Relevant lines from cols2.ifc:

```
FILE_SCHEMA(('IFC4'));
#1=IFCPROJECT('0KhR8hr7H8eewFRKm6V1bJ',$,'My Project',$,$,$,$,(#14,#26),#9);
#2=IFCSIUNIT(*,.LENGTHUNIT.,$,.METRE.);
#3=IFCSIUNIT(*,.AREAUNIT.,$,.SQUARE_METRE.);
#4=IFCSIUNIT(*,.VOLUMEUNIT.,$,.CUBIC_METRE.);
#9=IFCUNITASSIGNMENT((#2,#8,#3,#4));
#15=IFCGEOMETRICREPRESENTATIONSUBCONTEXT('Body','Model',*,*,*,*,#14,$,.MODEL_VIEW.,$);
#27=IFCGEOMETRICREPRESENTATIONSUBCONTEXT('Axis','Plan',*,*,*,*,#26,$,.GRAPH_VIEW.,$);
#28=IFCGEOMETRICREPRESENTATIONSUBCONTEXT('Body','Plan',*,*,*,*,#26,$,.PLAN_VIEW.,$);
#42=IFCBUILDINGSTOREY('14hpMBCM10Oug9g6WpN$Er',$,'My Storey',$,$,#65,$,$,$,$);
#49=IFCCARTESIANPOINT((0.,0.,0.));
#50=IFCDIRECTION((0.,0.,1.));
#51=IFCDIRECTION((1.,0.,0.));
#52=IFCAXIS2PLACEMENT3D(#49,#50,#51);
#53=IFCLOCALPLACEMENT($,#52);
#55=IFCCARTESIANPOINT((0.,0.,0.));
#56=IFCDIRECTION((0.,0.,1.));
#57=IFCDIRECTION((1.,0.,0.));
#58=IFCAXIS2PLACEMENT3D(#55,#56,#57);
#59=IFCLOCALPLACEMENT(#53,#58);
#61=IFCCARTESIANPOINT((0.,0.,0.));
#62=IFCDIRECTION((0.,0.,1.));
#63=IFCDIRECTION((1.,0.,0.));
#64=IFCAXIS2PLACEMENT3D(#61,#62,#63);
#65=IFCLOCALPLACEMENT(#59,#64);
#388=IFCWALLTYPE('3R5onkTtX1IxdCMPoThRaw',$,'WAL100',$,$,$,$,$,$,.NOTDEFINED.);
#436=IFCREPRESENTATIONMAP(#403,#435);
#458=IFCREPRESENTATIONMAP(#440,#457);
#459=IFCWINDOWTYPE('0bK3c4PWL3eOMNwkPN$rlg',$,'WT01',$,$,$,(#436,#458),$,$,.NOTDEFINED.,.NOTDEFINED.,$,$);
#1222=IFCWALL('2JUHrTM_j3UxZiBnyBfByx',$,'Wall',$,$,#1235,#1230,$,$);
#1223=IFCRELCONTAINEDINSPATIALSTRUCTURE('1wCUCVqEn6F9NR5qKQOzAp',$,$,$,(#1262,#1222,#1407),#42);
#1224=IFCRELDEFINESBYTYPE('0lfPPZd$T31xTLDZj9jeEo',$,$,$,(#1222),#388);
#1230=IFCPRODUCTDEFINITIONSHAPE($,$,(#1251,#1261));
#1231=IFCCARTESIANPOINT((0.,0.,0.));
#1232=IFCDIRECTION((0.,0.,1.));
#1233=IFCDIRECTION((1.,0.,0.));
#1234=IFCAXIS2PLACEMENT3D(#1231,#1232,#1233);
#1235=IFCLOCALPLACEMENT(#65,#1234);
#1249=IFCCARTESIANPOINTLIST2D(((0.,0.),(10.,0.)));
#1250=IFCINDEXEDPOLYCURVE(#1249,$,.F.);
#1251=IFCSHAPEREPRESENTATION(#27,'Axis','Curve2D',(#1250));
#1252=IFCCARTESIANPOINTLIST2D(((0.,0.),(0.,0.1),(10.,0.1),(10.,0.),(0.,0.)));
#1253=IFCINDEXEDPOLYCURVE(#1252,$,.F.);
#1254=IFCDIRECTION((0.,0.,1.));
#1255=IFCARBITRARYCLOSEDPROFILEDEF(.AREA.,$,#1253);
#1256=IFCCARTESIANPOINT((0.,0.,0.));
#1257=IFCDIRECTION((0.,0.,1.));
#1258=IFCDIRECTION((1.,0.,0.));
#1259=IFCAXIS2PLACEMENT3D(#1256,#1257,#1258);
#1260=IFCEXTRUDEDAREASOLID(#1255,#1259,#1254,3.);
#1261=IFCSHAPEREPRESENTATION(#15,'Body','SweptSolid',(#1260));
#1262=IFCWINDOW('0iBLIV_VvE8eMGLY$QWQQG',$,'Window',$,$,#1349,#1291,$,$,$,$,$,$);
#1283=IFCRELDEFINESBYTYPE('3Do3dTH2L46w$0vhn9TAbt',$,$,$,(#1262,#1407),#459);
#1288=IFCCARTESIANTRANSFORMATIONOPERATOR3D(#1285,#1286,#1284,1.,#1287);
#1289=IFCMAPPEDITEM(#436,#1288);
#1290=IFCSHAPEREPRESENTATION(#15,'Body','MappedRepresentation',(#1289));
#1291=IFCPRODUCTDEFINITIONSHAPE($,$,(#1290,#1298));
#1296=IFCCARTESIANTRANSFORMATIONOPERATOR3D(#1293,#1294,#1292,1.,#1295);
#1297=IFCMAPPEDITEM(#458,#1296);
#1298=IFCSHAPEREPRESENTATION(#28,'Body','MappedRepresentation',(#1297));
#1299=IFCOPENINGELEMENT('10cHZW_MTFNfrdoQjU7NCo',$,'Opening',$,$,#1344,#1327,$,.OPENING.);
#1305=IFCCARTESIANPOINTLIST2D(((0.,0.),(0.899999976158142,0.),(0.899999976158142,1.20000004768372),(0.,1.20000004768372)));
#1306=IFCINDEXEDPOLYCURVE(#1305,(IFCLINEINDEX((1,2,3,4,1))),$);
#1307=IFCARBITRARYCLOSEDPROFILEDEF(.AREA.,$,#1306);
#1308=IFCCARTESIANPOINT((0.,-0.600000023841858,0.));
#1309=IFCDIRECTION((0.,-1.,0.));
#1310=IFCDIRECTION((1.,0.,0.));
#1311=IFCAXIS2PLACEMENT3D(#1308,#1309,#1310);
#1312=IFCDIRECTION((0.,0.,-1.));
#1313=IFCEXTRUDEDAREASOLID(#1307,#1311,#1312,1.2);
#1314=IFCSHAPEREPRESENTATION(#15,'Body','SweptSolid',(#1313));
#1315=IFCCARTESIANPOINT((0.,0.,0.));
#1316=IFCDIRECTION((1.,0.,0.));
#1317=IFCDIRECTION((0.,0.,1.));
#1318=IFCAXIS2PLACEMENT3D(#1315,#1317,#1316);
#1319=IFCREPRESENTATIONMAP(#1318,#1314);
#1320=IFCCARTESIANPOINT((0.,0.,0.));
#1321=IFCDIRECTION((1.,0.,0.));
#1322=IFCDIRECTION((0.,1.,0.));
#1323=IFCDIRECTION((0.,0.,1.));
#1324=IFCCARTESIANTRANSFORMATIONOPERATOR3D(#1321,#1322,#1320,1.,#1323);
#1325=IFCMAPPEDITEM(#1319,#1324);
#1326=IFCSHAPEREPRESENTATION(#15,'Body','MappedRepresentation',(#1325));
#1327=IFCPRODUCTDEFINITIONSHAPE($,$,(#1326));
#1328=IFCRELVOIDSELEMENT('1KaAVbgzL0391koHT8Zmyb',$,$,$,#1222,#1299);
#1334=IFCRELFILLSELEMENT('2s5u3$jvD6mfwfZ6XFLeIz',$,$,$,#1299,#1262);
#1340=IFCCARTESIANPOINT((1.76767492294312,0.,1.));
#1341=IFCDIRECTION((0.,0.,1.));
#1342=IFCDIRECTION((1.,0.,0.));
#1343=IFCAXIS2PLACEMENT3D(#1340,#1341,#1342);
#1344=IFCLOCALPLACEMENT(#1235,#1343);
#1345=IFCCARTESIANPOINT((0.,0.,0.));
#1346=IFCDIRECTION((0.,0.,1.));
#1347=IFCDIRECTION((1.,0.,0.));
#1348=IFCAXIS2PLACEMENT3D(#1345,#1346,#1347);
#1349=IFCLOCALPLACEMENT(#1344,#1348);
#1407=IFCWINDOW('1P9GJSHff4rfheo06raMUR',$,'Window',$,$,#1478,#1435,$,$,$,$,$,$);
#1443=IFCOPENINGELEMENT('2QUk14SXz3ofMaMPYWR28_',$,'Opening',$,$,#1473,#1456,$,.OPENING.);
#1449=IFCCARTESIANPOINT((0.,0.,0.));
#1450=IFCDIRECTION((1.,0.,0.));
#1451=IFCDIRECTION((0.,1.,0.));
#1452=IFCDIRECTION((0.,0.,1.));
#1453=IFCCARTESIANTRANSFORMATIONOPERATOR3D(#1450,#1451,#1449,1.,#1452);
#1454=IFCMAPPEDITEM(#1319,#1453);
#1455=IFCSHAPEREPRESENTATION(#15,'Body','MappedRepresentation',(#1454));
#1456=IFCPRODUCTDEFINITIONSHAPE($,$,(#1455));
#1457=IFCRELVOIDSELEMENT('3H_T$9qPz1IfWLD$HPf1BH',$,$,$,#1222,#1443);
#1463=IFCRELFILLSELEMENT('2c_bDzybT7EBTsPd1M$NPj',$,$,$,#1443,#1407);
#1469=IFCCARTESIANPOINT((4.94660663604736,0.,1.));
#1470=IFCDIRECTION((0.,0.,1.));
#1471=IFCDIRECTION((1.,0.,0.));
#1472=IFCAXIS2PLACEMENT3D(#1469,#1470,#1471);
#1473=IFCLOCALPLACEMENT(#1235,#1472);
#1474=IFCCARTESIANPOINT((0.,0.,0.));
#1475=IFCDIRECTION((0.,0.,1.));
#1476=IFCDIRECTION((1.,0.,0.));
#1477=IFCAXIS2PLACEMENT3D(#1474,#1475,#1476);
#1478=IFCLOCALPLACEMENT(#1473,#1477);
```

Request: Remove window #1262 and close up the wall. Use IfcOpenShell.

```python
import ifcopenshell
import ifcopenshell.api.feature
import ifcopenshell.api.root
import ifcopenshell.geom
import ifcopenshell.util.shape

model = ifcopenshell.open("cols2.ifc")
settings = ifcopenshell.geom.settings()


def volume(element):
    """Net volume in cubic metres, openings subtracted."""
    shape = ifcopenshell.geom.create_shape(settings, element)
    return ifcopenshell.util.shape.get_volume(shape.geometry)


window = model.by_guid("0iBLIV_VvE8eMGLY$QWQQG")
opening = window.FillsVoids[0].RelatingOpeningElement
wall = opening.VoidsElements[0].RelatingBuildingElement
before = volume(wall)

ifcopenshell.api.root.remove_product(model, product=window)
ifcopenshell.api.feature.remove_feature(model, feature=opening)

after = volume(wall)

print(f"wall volume {before:.3f} -> {after:.3f} m3")

model.write("cols2_edited.ifc")
```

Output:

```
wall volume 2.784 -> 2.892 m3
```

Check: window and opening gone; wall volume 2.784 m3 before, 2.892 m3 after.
